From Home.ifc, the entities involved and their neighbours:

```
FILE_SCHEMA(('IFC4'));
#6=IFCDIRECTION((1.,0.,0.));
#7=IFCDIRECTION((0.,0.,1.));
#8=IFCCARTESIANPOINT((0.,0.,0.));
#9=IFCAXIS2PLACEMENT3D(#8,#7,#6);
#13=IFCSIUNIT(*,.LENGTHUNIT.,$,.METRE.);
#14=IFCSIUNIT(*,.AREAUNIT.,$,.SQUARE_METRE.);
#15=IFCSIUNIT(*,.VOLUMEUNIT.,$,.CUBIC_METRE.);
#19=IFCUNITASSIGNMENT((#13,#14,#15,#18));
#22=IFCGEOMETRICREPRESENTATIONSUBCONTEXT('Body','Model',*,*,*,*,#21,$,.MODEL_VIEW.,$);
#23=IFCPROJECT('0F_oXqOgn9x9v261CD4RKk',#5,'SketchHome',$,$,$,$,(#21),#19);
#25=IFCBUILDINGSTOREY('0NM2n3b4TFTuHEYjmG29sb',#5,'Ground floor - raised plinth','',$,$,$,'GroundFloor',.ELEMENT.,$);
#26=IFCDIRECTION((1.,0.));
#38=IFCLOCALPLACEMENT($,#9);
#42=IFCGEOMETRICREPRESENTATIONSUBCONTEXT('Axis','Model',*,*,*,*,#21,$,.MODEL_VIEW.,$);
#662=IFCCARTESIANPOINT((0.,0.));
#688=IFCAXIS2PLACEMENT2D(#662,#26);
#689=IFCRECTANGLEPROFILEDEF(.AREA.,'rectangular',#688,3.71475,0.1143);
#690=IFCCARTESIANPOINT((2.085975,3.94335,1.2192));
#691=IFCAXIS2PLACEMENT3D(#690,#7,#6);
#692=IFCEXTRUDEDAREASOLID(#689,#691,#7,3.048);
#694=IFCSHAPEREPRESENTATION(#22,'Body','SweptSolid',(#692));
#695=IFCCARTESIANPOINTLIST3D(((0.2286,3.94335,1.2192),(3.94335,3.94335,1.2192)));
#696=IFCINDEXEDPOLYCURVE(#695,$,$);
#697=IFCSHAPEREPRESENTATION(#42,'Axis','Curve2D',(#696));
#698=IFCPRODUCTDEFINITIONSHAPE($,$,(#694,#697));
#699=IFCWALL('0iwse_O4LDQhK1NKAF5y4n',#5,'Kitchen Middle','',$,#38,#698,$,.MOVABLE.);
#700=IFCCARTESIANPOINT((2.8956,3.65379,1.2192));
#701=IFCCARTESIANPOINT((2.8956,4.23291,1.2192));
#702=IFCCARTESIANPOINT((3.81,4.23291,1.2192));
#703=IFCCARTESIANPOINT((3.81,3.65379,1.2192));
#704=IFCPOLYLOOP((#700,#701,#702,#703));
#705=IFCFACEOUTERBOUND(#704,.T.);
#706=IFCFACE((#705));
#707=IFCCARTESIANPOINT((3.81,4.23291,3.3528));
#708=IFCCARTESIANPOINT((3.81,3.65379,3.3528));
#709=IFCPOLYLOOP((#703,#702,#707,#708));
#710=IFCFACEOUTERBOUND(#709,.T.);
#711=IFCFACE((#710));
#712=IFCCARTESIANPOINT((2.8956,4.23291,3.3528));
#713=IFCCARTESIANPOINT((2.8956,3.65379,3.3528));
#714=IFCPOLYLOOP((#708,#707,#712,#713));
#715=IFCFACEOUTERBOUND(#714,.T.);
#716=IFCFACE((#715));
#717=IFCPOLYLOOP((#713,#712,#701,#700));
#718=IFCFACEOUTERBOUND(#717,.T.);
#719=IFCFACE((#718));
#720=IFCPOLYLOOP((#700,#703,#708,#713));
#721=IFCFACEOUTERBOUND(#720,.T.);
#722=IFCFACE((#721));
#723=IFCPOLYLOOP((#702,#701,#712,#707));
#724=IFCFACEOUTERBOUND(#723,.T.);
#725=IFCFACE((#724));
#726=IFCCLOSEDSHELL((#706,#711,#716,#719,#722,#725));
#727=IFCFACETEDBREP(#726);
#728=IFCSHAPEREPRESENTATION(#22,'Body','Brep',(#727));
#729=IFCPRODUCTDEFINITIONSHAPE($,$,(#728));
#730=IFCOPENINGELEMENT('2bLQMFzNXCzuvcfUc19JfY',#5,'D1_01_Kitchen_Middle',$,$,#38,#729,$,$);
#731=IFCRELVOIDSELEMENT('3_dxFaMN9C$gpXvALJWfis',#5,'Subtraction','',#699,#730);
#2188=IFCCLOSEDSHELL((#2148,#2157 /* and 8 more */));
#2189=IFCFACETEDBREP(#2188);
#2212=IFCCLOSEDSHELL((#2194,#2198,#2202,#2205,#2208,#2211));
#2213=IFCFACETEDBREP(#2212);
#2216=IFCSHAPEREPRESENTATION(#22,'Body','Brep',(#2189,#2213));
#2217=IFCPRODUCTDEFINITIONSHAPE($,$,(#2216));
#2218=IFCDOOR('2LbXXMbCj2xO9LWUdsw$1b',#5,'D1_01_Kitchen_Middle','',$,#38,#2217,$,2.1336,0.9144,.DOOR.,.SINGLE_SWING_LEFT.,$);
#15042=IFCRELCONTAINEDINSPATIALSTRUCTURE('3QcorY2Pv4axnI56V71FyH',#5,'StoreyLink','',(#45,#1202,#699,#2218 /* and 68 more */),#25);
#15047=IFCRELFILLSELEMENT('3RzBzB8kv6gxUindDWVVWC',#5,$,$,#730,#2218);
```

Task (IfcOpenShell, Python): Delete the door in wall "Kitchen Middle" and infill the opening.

```python
import ifcopenshell
import ifcopenshell.api.feature
import ifcopenshell.api.root
import ifcopenshell.geom
import ifcopenshell.util.shape

model = ifcopenshell.open("Home.ifc")
settings = ifcopenshell.geom.settings()


def volume(element):
    """Net volume in cubic metres, openings subtracted."""
    shape = ifcopenshell.geom.create_shape(settings, element)
    return ifcopenshell.util.shape.get_volume(shape.geometry)


door = model.by_id(2218)
opening = door.FillsVoids[0].RelatingOpeningElement
wall = opening.VoidsElements[0].RelatingBuildingElement
before = volume(wall)

ifcopenshell.api.root.remove_product(model, product=door)
ifcopenshell.api.feature.remove_feature(model, feature=opening)

after = volume(wall)

print(f"wall volume {before:.3f} -> {after:.3f} m3")

model.write("Home_updated.ifc")
```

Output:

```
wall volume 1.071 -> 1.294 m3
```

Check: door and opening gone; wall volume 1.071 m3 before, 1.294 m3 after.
